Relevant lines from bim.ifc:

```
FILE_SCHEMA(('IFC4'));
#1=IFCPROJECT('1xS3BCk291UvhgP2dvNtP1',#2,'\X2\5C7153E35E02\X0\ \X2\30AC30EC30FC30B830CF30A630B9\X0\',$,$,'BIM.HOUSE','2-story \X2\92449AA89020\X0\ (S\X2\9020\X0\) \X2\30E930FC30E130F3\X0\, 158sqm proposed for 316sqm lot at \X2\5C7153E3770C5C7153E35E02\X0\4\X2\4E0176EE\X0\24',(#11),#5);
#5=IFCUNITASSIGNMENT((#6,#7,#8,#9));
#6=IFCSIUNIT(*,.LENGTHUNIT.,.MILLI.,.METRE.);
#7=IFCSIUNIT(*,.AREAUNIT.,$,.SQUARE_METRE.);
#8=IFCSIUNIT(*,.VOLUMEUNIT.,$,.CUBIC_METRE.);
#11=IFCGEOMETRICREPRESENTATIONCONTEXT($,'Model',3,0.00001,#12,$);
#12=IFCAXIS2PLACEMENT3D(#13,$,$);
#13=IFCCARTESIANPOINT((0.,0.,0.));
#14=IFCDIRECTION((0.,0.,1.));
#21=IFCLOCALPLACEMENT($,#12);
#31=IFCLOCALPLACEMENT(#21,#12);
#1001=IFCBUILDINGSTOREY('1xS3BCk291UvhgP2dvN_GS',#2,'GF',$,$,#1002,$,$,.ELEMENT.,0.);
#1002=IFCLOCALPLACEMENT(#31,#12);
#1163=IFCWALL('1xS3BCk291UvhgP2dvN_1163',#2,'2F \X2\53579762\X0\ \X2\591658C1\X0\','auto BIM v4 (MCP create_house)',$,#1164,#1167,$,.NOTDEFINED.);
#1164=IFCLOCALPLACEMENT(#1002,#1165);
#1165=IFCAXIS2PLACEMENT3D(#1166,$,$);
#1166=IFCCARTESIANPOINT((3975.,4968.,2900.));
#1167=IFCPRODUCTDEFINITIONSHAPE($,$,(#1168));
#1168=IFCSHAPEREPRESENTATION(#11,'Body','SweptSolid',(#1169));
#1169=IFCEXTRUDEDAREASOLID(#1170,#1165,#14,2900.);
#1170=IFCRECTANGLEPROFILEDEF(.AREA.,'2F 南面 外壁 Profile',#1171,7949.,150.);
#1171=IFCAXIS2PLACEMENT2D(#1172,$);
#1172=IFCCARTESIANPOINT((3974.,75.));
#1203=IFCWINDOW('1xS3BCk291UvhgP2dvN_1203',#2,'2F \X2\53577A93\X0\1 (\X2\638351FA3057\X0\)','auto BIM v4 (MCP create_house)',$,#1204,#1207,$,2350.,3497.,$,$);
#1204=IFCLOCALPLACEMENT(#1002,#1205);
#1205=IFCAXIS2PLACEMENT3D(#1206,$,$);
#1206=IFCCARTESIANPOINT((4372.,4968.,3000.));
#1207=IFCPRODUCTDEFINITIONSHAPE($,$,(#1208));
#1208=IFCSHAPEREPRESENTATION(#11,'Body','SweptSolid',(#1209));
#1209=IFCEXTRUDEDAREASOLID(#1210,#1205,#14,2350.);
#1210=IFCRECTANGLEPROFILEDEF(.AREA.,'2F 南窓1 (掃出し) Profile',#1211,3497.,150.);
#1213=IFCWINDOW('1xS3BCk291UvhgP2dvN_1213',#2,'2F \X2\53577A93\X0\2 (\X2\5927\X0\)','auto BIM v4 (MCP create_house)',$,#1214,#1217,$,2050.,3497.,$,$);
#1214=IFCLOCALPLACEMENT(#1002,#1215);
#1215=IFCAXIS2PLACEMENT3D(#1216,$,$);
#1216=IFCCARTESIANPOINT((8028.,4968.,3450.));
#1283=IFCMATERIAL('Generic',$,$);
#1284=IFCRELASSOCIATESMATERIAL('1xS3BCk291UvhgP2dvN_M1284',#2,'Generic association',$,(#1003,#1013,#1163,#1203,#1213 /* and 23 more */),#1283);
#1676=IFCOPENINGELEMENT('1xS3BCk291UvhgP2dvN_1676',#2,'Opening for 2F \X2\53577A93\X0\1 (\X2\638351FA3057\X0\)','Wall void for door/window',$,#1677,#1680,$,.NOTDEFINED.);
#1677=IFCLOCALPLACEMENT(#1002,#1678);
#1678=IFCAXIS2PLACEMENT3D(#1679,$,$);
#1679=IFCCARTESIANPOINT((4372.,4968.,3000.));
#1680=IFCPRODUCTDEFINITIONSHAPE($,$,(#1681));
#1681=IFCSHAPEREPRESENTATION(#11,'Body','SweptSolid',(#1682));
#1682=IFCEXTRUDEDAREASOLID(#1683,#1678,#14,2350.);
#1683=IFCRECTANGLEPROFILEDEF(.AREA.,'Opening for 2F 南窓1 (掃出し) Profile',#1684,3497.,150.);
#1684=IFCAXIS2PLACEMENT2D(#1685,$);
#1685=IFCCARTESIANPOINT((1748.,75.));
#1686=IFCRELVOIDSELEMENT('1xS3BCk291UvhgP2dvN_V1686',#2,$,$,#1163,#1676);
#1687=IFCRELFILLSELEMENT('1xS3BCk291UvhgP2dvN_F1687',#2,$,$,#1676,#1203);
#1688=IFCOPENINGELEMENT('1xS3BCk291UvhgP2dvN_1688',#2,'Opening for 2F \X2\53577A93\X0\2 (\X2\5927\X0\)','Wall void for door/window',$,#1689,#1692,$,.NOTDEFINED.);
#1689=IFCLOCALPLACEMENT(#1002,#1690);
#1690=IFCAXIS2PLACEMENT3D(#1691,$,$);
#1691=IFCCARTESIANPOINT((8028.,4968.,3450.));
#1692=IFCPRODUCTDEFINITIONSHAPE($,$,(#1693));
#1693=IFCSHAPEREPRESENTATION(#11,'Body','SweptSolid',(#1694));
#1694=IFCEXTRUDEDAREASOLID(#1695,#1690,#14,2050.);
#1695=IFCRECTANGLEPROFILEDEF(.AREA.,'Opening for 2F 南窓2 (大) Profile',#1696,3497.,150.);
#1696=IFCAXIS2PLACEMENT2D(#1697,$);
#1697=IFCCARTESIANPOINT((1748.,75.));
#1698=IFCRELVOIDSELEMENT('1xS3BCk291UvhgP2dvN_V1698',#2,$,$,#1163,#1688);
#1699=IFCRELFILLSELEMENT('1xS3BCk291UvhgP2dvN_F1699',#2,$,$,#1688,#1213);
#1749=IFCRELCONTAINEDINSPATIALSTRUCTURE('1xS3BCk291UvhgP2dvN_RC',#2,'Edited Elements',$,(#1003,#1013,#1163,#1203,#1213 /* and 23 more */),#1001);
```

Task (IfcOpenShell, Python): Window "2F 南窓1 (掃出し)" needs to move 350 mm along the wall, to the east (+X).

```python
import ifcopenshell
import ifcopenshell.api.geometry
import ifcopenshell.util.placement
import ifcopenshell.util.unit

model = ifcopenshell.open("bim.ifc")
unit_scale = ifcopenshell.util.unit.calculate_unit_scale(model)

window = model.by_guid("1xS3BCk291UvhgP2dvN_1203")
opening = window.FillsVoids[0].RelatingOpeningElement
wall = opening.VoidsElements[0].RelatingBuildingElement

wall_matrix = ifcopenshell.util.placement.get_local_placement(wall.ObjectPlacement)
shift = wall_matrix[:3, 0] * 0.35 / unit_scale
before = ifcopenshell.util.placement.get_local_placement(window.ObjectPlacement)[:3, 3].copy()

# The window is not placed relative to its opening, so move both.
for product in (opening, window):
    matrix = ifcopenshell.util.placement.get_local_placement(product.ObjectPlacement)
    matrix[:3, 3] += shift
    ifcopenshell.api.geometry.edit_object_placement(model, product=product, matrix=matrix, is_si=False)

after = ifcopenshell.util.placement.get_local_placement(window.ObjectPlacement)[:3, 3]
print("window moved by", (after - before).round(3) + 0.0)

model.write("bim_edited.ifc")
```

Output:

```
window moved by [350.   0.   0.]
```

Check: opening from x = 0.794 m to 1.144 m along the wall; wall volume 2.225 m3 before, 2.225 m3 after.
